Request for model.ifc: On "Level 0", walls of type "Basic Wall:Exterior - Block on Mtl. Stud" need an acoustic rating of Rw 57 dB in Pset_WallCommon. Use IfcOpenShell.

First a look at what the model holds.

```python
import ifcopenshell
import ifcopenshell.util.element

model = ifcopenshell.open("model.ifc")
print(model.schema)
storey = next(s for s in model.by_type("IfcBuildingStorey") if s.Name == "Level 0")
walls = [e for e in ifcopenshell.util.element.get_decomposition(storey) if e.is_a("IfcWall")]
seen = {}
for e in walls:
    element_type = ifcopenshell.util.element.get_type(e)
    key = (element_type.Name if element_type != e and element_type else None, ifcopenshell.util.element.get_pset(e, "Pset_WallCommon", "AcousticRating"))
    seen[key] = seen.get(key, 0) + 1
for (name, value), count in sorted(seen.items(), key=str):
    print(count, "x", name, "|", value)
```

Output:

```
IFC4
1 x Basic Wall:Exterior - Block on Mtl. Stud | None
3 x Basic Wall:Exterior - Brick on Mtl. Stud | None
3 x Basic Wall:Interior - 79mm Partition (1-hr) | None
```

```python
import ifcopenshell
import ifcopenshell.api.pset
import ifcopenshell.util.element

model = ifcopenshell.open("model.ifc")

storey = next(s for s in model.by_type("IfcBuildingStorey") if s.Name == "Level 0")
walls = [e for e in ifcopenshell.util.element.get_decomposition(storey) if e.is_a("IfcWall")]

count = 0
for e in walls:
    element_type = ifcopenshell.util.element.get_type(e)
    if element_type in (None, e) or element_type.Name != "Basic Wall:Exterior - Block on Mtl. Stud":
        continue
    # add_pset returns the element's existing set when there is one.
    pset = ifcopenshell.api.pset.add_pset(model, product=e, name="Pset_WallCommon")
    ifcopenshell.api.pset.edit_pset(model, pset=pset, properties={"AcousticRating": "Rw 57 dB"})
    count += 1

print(count, "walls updated")

model.write("model_updated.ifc")
```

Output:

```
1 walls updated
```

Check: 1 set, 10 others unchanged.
